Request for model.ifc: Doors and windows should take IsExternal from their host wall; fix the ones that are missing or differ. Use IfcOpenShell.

First a look at what the model holds.

```python
import ifcopenshell
import ifcopenshell.util.element

model = ifcopenshell.open("model.ifc")
print(model.schema)
seen = {}
for e in model.by_type("IfcDoor") + model.by_type("IfcWindow"):
    if not e.FillsVoids:
        continue
    host = e.FillsVoids[0].RelatingOpeningElement.VoidsElements[0].RelatingBuildingElement
    own = ifcopenshell.util.element.get_pset(e, f"Pset_{e.is_a()[3:].removesuffix('StandardCase')}Common", "IsExternal")
    wall = ifcopenshell.util.element.get_pset(host, "Pset_WallCommon", "IsExternal")
    seen[e.is_a(), own, wall] = seen.get((e.is_a(), own, wall), 0) + 1
for (cls, own, wall), count in sorted(seen.items(), key=str):
    print(count, cls, "IsExternal:", own, "| host wall:", wall)
```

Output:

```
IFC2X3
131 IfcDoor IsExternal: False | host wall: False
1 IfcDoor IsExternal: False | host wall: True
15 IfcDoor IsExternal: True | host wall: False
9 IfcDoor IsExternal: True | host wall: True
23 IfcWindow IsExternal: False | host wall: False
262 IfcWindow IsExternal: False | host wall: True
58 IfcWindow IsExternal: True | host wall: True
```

```python
import ifcopenshell
import ifcopenshell.api.pset
import ifcopenshell.util.element

model = ifcopenshell.open("model.ifc")

count = 0
for ifc_class, pset_name in (("IfcDoor", "Pset_DoorCommon"), ("IfcWindow", "Pset_WindowCommon")):
    for e in model.by_type(ifc_class):
        if not e.FillsVoids:
            continue
        host = e.FillsVoids[0].RelatingOpeningElement.VoidsElements[0].RelatingBuildingElement
        external = ifcopenshell.util.element.get_pset(host, "Pset_WallCommon", "IsExternal")
        if external is None or ifcopenshell.util.element.get_pset(e, pset_name, "IsExternal") == external:
            continue
        pset = ifcopenshell.api.pset.add_pset(model, product=e, name=pset_name)
        ifcopenshell.api.pset.edit_pset(model, pset=pset, properties={"IsExternal": external})
        count += 1

print(count, "updated")

model.write("model_updated.ifc")
```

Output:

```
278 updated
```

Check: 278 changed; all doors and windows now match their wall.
